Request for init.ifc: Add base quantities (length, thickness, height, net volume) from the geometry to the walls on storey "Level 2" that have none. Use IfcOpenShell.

First a look at what the model holds.

```python
import ifcopenshell
import ifcopenshell.util.element
import ifcopenshell.util.unit

model = ifcopenshell.open("init.ifc")
print(model.schema)
for unit_type in ("LENGTHUNIT", "AREAUNIT", "VOLUMEUNIT"):
    print(unit_type, ifcopenshell.util.unit.calculate_unit_scale(model, unit_type))
storey = next(s for s in model.by_type("IfcBuildingStorey") if s.Name == "Level 2")
walls = [e for e in ifcopenshell.util.element.get_decomposition(storey) if e.is_a("IfcWall")]
for e in sorted(walls, key=lambda e: e.id()):
    print(e.id(), e.is_a(), e.Name, list(ifcopenshell.util.element.get_psets(e, qtos_only=True)), sep=" | ")
```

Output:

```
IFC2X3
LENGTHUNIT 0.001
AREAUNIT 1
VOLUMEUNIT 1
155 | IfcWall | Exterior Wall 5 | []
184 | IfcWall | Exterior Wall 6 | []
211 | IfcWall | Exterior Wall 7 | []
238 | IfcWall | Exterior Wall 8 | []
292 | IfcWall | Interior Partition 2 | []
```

```python
import ifcopenshell
import ifcopenshell.api.pset
import ifcopenshell.geom
import ifcopenshell.util.element
import ifcopenshell.util.shape
import ifcopenshell.util.unit

model = ifcopenshell.open("init.ifc")
unit_scale = ifcopenshell.util.unit.calculate_unit_scale(model)
volume_scale = ifcopenshell.util.unit.calculate_unit_scale(model, "VOLUMEUNIT")
settings = ifcopenshell.geom.settings()

storey = next(s for s in model.by_type("IfcBuildingStorey") if s.Name == "Level 2")
walls = [e for e in ifcopenshell.util.element.get_decomposition(storey) if e.is_a("IfcWall")]

for e in sorted(walls, key=lambda e: e.id()):
    if ifcopenshell.util.element.get_psets(e, qtos_only=True, should_inherit=False):
        continue
    # Geometry comes back in metres, in the element's own axes.
    shape = ifcopenshell.geom.create_shape(settings, e)
    values = {
        "Length": ifcopenshell.util.shape.get_x(shape.geometry) / unit_scale,
        "Width": ifcopenshell.util.shape.get_y(shape.geometry) / unit_scale,
        "Height": ifcopenshell.util.shape.get_z(shape.geometry) / unit_scale,
        "NetVolume": ifcopenshell.util.shape.get_volume(shape.geometry) / volume_scale,
    }
    qto = ifcopenshell.api.pset.add_qto(model, product=e, name="BaseQuantities")
    ifcopenshell.api.pset.edit_qto(model, qto=qto, properties=values)
    print(e.id(), {k: round(v, 3) for k, v in values.items()})

model.write("init_edited.ifc")
```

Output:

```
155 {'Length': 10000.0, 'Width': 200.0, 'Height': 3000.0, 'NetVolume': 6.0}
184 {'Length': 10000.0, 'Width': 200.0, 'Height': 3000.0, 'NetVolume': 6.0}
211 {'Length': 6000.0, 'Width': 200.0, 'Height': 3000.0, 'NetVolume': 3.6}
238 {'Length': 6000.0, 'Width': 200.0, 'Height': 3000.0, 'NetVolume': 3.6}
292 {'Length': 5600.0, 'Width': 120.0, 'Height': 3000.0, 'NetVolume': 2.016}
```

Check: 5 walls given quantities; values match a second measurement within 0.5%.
